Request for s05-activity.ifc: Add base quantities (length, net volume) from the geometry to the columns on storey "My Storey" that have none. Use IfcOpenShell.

First a look at what the model holds.

```python
import ifcopenshell
import ifcopenshell.util.element
import ifcopenshell.util.unit

model = ifcopenshell.open("s05-activity.ifc")
print(model.schema)
for unit_type in ("LENGTHUNIT", "AREAUNIT", "VOLUMEUNIT"):
    print(unit_type, ifcopenshell.util.unit.calculate_unit_scale(model, unit_type))
storey = next(s for s in model.by_type("IfcBuildingStorey") if s.Name == "My Storey")
columns = [e for e in ifcopenshell.util.element.get_decomposition(storey) if e.is_a("IfcColumn")]
for e in sorted(columns, key=lambda e: e.id()):
    print(e.id(), e.is_a(), e.Name, list(ifcopenshell.util.element.get_psets(e, qtos_only=True)), sep=" | ")
```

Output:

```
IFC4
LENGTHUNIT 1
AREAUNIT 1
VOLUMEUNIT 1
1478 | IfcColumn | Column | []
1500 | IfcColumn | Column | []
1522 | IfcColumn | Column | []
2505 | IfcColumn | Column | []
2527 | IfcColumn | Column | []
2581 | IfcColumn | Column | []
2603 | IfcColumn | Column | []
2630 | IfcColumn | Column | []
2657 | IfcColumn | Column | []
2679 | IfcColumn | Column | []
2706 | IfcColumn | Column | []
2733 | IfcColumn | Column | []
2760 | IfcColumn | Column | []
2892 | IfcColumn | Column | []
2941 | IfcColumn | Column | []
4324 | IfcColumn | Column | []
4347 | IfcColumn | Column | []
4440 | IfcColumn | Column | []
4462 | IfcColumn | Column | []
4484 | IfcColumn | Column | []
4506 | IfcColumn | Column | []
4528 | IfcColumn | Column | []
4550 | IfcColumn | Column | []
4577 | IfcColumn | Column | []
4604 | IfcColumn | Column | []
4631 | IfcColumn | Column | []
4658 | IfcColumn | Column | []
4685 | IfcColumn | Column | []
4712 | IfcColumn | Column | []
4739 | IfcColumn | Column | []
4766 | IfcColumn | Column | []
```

```python
import ifcopenshell
import ifcopenshell.api.pset
import ifcopenshell.geom
import ifcopenshell.util.element
import ifcopenshell.util.shape
import ifcopenshell.util.unit

model = ifcopenshell.open("s05-activity.ifc")
unit_scale = ifcopenshell.util.unit.calculate_unit_scale(model)
volume_scale = ifcopenshell.util.unit.calculate_unit_scale(model, "VOLUMEUNIT")
settings = ifcopenshell.geom.settings()

storey = next(s for s in model.by_type("IfcBuildingStorey") if s.Name == "My Storey")
columns = [e for e in ifcopenshell.util.element.get_decomposition(storey) if e.is_a("IfcColumn")]

for e in sorted(columns, key=lambda e: e.id()):
    if ifcopenshell.util.element.get_psets(e, qtos_only=True, should_inherit=False):
        continue
    # Geometry comes back in metres, in the element's own axes.
    shape = ifcopenshell.geom.create_shape(settings, e)
    values = {
        "Length": ifcopenshell.util.shape.get_z(shape.geometry) / unit_scale,
        "NetVolume": ifcopenshell.util.shape.get_volume(shape.geometry) / volume_scale,
    }
    qto = ifcopenshell.api.pset.add_qto(model, product=e, name="Qto_ColumnBaseQuantities")
    ifcopenshell.api.pset.edit_qto(model, qto=qto, properties=values)
    print(e.id(), {k: round(v, 3) for k, v in values.items()})

model.write("s05-activity-out.ifc")
```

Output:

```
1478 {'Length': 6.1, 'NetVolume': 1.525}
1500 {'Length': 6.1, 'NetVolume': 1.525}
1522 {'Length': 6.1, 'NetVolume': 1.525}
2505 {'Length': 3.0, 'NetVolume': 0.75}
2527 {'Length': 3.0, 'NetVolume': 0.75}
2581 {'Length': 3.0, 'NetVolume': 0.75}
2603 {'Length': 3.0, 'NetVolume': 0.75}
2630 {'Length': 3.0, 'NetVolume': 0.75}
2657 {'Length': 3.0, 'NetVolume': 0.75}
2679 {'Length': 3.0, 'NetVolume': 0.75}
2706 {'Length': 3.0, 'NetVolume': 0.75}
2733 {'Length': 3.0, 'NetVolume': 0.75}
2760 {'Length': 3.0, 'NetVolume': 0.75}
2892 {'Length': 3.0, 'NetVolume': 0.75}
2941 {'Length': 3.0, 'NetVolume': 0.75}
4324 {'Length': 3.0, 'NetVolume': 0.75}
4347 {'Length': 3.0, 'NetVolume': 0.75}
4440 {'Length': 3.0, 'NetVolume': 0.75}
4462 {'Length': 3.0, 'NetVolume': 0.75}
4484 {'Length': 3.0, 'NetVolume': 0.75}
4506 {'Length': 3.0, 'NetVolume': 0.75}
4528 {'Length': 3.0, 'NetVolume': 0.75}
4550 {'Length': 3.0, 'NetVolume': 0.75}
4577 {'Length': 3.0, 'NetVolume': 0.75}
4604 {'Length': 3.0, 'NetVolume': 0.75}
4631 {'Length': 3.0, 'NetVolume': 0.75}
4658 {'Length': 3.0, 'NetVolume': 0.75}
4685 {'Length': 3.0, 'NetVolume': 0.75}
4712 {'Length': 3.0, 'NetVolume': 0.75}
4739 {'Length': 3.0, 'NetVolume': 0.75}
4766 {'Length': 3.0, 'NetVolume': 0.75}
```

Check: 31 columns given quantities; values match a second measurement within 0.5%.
